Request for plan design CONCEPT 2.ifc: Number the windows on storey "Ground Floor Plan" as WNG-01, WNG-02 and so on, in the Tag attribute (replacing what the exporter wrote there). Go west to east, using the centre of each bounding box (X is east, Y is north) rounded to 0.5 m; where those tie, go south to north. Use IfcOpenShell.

First a look at what the model holds.

```python
import ifcopenshell
import ifcopenshell.util.element
import ifcopenshell.util.placement

model = ifcopenshell.open("plan design CONCEPT 2.ifc")
print(model.schema)
storey = next(s for s in model.by_type("IfcBuildingStorey") if s.Name == "Ground Floor Plan")
windows = [e for e in ifcopenshell.util.element.get_decomposition(storey) if e.is_a("IfcWindow")]
for e in sorted(windows, key=lambda e: e.id()):
    origin = ifcopenshell.util.placement.get_local_placement(e.ObjectPlacement)[:3, 3]
    print(e.id(), e.Tag, e.Name, origin.round(2) + 0.0, sep=" | ")
```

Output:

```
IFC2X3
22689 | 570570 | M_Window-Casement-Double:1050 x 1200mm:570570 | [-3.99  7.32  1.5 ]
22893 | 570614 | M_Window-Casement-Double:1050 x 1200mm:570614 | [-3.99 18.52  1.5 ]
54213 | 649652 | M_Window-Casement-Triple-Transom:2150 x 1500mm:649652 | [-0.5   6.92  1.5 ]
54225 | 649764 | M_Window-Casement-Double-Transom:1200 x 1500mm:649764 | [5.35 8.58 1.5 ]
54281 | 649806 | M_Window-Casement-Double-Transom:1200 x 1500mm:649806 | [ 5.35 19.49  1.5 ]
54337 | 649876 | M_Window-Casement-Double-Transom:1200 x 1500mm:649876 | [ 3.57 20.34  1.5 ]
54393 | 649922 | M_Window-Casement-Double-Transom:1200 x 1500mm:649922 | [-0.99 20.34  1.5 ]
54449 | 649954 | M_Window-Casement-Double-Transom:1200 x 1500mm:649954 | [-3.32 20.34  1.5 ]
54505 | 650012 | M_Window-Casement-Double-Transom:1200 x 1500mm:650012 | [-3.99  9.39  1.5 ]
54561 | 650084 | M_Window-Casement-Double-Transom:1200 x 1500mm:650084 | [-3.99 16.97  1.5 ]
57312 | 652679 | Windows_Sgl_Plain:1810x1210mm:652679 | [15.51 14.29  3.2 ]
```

```python
import ifcopenshell
import ifcopenshell.geom
import ifcopenshell.util.element
import ifcopenshell.util.shape

model = ifcopenshell.open("plan design CONCEPT 2.ifc")
settings = ifcopenshell.geom.settings()
settings.set("use-world-coords", True)


def centre(element):
    shape = ifcopenshell.geom.create_shape(settings, element)
    return ifcopenshell.util.shape.get_bbox_centroid(shape.geometry)


storey = next(s for s in model.by_type("IfcBuildingStorey") if s.Name == "Ground Floor Plan")
windows = [e for e in ifcopenshell.util.element.get_decomposition(storey) if e.is_a("IfcWindow")]

# Insertion points can sit at a corner or the storey origin, so sort by the geometry (in metres).
centres = {e: centre(e) for e in windows}
windows.sort(key=lambda e: (round(centres[e][0] / 0.5), centres[e][1]))

for i, e in enumerate(windows, start=1):
    number = f"WNG-{i:02d}"
    e.Tag = number
    print(e.id(), number)

model.write("plan design CONCEPT 2-out.ifc")
```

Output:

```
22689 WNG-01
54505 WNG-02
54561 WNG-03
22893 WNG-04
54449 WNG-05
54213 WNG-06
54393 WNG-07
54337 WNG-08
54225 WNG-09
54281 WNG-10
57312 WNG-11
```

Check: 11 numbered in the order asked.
